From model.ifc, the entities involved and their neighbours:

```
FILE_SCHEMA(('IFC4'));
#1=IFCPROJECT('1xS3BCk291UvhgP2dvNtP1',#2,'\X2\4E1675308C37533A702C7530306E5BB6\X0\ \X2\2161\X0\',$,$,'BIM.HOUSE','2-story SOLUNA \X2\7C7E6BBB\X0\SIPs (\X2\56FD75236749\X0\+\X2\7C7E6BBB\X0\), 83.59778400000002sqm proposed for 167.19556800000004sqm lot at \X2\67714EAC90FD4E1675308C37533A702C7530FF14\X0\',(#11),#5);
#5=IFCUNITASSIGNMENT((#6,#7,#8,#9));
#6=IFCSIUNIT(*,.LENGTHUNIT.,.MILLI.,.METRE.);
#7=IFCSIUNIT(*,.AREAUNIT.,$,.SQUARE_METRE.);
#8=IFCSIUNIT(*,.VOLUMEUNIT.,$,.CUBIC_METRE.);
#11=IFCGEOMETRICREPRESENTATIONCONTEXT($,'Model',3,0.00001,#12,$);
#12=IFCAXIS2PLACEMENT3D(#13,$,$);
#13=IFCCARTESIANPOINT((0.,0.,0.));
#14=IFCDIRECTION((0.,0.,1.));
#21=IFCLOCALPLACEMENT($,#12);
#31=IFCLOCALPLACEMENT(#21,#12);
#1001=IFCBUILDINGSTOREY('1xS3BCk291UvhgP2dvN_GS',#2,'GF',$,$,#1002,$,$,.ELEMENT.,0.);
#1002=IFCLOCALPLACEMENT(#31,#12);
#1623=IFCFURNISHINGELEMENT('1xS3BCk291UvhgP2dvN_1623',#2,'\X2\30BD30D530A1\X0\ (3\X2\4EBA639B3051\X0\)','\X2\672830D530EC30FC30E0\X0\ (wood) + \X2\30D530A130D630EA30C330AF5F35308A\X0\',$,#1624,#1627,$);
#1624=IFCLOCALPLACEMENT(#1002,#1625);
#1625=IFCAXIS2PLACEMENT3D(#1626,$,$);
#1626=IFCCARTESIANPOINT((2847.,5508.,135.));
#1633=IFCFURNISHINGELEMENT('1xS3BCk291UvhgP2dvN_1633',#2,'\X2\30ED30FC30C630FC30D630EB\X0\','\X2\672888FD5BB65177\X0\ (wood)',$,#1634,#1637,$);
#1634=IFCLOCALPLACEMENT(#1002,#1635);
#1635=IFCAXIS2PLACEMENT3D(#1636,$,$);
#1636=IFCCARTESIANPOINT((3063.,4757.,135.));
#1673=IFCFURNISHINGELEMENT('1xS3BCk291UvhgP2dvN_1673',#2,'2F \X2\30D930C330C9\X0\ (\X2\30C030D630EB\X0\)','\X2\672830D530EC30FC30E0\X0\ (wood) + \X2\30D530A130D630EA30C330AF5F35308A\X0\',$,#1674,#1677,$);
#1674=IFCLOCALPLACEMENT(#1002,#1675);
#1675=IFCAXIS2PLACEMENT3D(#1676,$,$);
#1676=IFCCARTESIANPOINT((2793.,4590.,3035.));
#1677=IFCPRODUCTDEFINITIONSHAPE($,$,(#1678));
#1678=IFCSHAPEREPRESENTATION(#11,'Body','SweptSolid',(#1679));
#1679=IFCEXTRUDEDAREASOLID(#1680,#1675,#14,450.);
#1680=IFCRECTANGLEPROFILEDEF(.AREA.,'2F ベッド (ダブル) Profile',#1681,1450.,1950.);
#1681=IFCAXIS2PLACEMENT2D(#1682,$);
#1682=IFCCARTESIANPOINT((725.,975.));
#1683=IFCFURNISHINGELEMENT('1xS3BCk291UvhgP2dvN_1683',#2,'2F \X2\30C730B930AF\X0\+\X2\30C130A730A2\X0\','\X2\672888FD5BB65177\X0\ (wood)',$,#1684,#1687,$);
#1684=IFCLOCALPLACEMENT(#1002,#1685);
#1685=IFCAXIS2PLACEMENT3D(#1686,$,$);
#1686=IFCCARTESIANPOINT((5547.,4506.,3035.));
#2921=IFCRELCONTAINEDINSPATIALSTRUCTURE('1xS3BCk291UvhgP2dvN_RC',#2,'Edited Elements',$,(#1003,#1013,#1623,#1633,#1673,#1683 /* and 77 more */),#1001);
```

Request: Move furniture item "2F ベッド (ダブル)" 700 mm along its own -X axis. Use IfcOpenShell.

```python
import ifcopenshell
import ifcopenshell.api.geometry
import ifcopenshell.util.placement
import ifcopenshell.util.unit

model = ifcopenshell.open("model.ifc")
unit_scale = ifcopenshell.util.unit.calculate_unit_scale(model)

item = model.by_guid("1xS3BCk291UvhgP2dvN_1673")
matrix = ifcopenshell.util.placement.get_local_placement(item.ObjectPlacement)
matrix[:3, 3] -= matrix[:3, 0] * 0.7 / unit_scale
ifcopenshell.api.geometry.edit_object_placement(model, product=item, matrix=matrix, is_si=False)

print(ifcopenshell.util.placement.get_local_placement(item.ObjectPlacement).round(3) + 0.0)

model.write("model-out.ifc")
```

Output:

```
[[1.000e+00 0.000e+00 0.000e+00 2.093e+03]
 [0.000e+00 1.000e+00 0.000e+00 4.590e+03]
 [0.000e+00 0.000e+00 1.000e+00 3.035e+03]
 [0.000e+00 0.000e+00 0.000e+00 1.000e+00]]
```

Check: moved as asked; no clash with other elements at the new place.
